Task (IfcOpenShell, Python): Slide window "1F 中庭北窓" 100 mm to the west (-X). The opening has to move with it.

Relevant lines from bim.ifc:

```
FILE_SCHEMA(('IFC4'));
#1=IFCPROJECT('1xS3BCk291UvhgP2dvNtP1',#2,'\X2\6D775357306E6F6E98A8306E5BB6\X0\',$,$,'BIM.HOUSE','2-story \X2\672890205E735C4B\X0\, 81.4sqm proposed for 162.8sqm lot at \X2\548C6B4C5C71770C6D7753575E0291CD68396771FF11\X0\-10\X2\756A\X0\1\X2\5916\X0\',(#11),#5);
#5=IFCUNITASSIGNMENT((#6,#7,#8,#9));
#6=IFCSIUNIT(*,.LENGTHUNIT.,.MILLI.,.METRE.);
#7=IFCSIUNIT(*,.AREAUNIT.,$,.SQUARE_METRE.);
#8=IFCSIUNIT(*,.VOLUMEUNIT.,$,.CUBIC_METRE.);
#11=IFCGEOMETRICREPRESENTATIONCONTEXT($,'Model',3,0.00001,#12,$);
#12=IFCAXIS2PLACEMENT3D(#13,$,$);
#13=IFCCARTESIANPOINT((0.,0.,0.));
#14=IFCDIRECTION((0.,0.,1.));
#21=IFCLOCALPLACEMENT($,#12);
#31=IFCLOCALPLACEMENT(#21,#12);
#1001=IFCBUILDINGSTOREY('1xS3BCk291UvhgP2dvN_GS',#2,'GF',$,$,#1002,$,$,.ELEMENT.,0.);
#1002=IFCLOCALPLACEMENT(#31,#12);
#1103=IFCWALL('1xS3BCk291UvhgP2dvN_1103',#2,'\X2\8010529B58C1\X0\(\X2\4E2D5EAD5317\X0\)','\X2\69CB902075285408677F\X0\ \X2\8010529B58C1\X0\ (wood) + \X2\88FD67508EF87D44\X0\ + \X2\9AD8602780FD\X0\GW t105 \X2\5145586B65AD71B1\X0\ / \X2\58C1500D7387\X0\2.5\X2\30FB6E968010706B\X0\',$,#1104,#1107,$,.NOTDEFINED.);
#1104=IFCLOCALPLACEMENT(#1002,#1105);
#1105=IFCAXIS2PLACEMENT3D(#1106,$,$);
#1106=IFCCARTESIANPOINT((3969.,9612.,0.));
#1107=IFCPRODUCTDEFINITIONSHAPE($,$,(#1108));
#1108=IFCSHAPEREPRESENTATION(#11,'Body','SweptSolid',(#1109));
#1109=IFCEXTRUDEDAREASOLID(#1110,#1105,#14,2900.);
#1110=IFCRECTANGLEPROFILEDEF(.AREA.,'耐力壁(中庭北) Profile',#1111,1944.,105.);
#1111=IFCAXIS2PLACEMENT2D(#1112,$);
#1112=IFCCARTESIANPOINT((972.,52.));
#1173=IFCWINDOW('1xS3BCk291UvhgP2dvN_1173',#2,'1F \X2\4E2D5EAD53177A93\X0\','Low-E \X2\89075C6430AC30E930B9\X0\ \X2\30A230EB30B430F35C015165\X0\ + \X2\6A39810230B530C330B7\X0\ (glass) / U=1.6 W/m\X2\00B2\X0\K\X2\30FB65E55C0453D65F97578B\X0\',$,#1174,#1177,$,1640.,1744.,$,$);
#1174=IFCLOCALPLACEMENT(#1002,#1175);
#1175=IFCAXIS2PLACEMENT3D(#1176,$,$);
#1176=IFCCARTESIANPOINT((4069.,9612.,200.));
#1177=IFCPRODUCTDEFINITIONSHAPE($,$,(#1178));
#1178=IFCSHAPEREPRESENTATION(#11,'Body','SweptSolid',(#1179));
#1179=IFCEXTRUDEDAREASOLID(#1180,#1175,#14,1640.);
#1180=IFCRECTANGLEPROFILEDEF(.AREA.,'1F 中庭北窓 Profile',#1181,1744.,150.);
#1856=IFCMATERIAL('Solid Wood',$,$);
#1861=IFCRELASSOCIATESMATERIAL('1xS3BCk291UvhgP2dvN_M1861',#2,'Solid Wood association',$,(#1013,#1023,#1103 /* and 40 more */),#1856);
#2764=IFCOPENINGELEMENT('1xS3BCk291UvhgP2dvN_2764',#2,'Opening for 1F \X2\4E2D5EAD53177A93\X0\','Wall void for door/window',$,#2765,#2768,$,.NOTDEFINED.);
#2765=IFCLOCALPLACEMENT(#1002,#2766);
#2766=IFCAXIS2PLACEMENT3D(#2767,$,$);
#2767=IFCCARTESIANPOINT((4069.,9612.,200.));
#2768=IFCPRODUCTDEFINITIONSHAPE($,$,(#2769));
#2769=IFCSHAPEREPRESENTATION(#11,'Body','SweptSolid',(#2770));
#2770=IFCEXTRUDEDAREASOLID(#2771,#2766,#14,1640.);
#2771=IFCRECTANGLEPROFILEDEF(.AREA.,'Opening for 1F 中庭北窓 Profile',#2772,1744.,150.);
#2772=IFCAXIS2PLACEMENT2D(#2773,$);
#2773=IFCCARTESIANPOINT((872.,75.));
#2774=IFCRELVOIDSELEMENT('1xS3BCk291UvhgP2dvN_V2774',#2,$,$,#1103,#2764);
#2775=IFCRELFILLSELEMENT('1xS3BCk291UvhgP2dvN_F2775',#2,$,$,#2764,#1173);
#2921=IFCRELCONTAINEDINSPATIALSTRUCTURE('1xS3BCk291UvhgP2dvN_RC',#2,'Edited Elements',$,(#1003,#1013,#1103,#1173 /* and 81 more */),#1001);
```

```python
import ifcopenshell
import ifcopenshell.api.geometry
import ifcopenshell.util.placement
import ifcopenshell.util.unit

model = ifcopenshell.open("bim.ifc")
unit_scale = ifcopenshell.util.unit.calculate_unit_scale(model)

window = model.by_guid("1xS3BCk291UvhgP2dvN_1173")
opening = window.FillsVoids[0].RelatingOpeningElement
wall = opening.VoidsElements[0].RelatingBuildingElement

wall_matrix = ifcopenshell.util.placement.get_local_placement(wall.ObjectPlacement)
shift = wall_matrix[:3, 0] * -0.1 / unit_scale
before = ifcopenshell.util.placement.get_local_placement(window.ObjectPlacement)[:3, 3].copy()

# The window is not placed relative to its opening, so move both.
for product in (opening, window):
    matrix = ifcopenshell.util.placement.get_local_placement(product.ObjectPlacement)
    matrix[:3, 3] += shift
    ifcopenshell.api.geometry.edit_object_placement(model, product=product, matrix=matrix, is_si=False)

after = ifcopenshell.util.placement.get_local_placement(window.ObjectPlacement)[:3, 3]
print("window moved by", (after - before).round(3) + 0.0)

model.write("bim_updated.ifc")
```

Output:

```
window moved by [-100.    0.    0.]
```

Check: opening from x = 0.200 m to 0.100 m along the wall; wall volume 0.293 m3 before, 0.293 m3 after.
